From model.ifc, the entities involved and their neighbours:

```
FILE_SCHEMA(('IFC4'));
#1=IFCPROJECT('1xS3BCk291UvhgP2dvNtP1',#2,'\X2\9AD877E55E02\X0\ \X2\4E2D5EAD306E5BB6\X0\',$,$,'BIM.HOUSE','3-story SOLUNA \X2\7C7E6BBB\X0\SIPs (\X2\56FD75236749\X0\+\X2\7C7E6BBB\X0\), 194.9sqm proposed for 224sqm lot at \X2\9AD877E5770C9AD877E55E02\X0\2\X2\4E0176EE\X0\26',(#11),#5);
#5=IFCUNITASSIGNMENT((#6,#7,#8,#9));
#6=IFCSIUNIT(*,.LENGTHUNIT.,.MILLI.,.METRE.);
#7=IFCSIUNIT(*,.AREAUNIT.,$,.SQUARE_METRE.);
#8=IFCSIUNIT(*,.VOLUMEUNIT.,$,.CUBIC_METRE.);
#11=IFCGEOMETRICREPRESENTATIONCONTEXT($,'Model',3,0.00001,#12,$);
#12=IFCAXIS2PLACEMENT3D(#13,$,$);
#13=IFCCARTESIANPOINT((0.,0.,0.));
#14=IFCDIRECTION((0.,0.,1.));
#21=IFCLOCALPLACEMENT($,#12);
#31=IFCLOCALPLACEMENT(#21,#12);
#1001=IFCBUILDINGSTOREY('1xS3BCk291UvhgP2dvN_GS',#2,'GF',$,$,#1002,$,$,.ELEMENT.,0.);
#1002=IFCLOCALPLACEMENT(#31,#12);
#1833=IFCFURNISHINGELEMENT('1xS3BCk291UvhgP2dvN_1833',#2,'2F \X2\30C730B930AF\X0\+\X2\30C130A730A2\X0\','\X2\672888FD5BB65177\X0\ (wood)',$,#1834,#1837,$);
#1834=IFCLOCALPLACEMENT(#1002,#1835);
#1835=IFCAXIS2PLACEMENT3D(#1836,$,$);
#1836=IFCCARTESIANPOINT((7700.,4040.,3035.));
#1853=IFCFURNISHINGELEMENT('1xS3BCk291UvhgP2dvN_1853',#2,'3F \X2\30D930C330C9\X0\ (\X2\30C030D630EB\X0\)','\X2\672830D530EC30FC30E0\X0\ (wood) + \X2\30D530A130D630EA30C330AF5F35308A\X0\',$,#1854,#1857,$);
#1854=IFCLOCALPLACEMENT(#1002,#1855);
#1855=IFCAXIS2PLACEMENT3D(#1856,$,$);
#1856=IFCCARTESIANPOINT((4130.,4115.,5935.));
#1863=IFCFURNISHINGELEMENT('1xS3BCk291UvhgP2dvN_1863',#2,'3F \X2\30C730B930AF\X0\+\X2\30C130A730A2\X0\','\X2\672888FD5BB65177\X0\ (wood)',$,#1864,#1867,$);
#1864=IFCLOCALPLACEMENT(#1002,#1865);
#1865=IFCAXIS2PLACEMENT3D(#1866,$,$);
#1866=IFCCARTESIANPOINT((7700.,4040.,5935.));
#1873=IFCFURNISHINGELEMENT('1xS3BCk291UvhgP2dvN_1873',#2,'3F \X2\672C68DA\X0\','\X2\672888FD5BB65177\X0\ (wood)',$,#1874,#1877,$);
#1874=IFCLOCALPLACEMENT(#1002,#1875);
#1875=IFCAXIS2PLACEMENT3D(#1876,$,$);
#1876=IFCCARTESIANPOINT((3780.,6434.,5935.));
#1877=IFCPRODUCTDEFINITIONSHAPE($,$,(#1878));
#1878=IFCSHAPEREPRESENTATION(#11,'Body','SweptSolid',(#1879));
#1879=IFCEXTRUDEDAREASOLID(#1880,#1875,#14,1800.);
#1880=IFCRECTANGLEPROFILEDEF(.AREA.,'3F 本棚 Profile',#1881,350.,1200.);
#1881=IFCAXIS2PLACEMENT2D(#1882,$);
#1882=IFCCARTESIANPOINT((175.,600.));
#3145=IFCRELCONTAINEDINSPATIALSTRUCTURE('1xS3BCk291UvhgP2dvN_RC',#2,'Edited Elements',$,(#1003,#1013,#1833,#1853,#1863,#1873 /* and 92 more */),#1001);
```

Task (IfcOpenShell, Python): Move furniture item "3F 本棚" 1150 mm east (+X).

```python
import ifcopenshell
import ifcopenshell.api.geometry
import ifcopenshell.util.placement
import ifcopenshell.util.unit

model = ifcopenshell.open("model.ifc")
unit_scale = ifcopenshell.util.unit.calculate_unit_scale(model)

item = model.by_guid("1xS3BCk291UvhgP2dvN_1873")
matrix = ifcopenshell.util.placement.get_local_placement(item.ObjectPlacement)
matrix[0, 3] += 1.15 / unit_scale
ifcopenshell.api.geometry.edit_object_placement(model, product=item, matrix=matrix, is_si=False)

print(ifcopenshell.util.placement.get_local_placement(item.ObjectPlacement).round(3) + 0.0)

model.write("model_v2.ifc")
```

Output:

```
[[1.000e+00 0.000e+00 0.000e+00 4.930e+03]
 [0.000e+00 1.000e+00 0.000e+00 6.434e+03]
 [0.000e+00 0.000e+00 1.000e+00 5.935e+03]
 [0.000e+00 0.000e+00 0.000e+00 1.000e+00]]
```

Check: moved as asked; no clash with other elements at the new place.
